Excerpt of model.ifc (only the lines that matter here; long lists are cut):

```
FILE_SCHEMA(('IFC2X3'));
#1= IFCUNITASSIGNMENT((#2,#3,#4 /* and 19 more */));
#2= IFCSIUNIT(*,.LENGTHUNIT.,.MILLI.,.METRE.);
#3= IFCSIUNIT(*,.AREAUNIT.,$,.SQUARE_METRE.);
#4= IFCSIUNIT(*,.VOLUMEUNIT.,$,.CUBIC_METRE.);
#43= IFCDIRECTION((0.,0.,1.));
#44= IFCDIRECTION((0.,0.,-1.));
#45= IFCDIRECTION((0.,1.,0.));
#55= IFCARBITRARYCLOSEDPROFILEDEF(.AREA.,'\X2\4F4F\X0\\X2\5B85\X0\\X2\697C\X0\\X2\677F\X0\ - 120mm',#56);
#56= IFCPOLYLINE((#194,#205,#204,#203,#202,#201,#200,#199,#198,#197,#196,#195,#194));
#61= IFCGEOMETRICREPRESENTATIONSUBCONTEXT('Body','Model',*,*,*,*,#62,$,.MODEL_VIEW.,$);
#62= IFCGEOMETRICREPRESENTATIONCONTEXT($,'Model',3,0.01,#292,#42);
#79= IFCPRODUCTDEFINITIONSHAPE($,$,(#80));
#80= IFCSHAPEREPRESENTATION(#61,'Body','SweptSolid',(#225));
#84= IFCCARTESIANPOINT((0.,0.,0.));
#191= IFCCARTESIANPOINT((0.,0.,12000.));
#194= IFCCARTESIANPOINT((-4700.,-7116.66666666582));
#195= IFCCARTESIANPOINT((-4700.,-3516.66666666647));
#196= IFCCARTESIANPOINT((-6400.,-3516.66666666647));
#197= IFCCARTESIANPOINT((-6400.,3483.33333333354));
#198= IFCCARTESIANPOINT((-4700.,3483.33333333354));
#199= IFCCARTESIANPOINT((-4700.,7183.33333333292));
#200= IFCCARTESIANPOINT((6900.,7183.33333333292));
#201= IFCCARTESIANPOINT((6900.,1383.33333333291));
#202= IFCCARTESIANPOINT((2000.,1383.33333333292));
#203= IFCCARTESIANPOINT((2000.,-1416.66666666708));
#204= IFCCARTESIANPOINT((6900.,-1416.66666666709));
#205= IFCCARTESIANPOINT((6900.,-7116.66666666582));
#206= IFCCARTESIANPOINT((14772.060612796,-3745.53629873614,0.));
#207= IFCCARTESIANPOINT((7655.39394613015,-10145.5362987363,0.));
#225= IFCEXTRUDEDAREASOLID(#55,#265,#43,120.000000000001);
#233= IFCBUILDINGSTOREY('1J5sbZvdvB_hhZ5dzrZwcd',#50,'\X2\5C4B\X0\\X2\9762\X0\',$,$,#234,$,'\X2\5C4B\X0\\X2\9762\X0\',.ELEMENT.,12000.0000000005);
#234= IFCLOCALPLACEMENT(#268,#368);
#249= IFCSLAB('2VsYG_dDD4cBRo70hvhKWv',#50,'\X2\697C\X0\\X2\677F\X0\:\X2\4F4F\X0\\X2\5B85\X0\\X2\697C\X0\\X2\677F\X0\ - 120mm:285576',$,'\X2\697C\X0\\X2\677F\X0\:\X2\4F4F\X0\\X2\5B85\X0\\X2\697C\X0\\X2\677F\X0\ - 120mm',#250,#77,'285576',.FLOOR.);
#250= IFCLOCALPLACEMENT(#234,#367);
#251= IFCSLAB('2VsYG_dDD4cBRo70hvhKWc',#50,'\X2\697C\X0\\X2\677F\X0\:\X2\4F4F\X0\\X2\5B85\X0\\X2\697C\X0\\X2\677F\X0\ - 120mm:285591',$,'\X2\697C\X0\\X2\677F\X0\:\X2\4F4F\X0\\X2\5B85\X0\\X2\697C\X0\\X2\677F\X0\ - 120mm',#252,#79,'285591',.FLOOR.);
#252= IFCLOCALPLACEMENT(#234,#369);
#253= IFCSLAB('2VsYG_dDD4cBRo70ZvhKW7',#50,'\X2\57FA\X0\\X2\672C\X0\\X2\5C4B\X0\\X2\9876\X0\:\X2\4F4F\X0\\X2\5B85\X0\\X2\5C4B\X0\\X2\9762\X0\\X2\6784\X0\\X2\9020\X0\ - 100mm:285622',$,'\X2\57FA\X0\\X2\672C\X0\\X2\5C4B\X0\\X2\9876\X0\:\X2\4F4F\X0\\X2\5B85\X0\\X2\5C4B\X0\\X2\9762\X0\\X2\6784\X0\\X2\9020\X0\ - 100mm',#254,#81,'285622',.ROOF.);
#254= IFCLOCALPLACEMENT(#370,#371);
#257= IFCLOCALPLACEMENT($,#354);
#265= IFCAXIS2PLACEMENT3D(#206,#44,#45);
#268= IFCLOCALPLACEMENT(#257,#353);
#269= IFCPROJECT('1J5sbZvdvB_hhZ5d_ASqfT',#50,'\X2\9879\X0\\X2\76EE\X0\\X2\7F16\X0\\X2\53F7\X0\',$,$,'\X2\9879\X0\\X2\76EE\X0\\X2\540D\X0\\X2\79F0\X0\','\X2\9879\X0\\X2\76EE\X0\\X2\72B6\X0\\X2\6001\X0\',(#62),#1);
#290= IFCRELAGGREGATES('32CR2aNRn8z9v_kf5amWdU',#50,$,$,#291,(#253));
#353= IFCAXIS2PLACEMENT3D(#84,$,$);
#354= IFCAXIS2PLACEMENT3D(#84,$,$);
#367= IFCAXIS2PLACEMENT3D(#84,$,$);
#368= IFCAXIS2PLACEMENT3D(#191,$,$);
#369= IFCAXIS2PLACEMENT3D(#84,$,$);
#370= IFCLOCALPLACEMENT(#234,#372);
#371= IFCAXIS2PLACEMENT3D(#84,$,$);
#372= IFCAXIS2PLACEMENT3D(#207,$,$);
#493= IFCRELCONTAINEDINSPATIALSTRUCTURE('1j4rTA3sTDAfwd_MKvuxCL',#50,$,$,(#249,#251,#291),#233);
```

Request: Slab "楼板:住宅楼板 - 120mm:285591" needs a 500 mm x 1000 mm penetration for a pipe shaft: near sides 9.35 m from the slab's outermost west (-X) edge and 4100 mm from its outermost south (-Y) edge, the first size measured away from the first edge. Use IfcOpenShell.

```python
import numpy as np
import ifcopenshell
import ifcopenshell.api.feature
import ifcopenshell.api.geometry
import ifcopenshell.api.root
import ifcopenshell.geom
import ifcopenshell.util.placement
import ifcopenshell.util.representation
import ifcopenshell.util.shape
import ifcopenshell.util.unit

model = ifcopenshell.open("model.ifc")
unit_scale = ifcopenshell.util.unit.calculate_unit_scale(model)
settings = ifcopenshell.geom.settings()


def volume(element):
    """Net volume in cubic metres, openings subtracted."""
    shape = ifcopenshell.geom.create_shape(settings, element)
    return ifcopenshell.util.shape.get_volume(shape.geometry)


slab = model.by_guid("2VsYG_dDD4cBRo70hvhKWc")
before = volume(slab)

# Extent in the slab's own axes, in metres. The edges named are its -X and -Y sides.
slab_shape = ifcopenshell.geom.create_shape(settings, slab)
vertices = ifcopenshell.util.shape.get_vertices(slab_shape.geometry)
x_min, y_min, bottom = vertices.min(axis=0)
top = vertices[:, 2].max()

opening = ifcopenshell.api.root.create_entity(model, ifc_class="IfcOpeningElement", name="Pipe shaft opening")
context = ifcopenshell.util.representation.get_context(model, "Model", "Body", "MODEL_VIEW")
width, depth = 0.5, 1
outline = [(0.0, 0.0), (width, 0.0), (width, depth), (0.0, depth), (0.0, 0.0)]
# Overshoot both faces by 50 mm so the cut is clean.
shape = ifcopenshell.api.geometry.add_slab_representation(
    model, context=context, depth=top - bottom + 0.1, polyline=outline
)
ifcopenshell.api.geometry.assign_representation(model, product=opening, representation=shape)

matrix = ifcopenshell.util.placement.get_local_placement(slab.ObjectPlacement)
matrix[:, 3] = matrix @ np.append(np.array([x_min + 9.35, y_min + 4.1, bottom - 0.05]) / unit_scale, 1.0)
ifcopenshell.api.geometry.edit_object_placement(model, product=opening, matrix=matrix, is_si=False)
ifcopenshell.api.feature.add_feature(model, feature=opening, element=slab)

after = volume(slab)

print(f"slab volume {before:.3f} -> {after:.3f} m3")

model.write("model_edited.ifc")
```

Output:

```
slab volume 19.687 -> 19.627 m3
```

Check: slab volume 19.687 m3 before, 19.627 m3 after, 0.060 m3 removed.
